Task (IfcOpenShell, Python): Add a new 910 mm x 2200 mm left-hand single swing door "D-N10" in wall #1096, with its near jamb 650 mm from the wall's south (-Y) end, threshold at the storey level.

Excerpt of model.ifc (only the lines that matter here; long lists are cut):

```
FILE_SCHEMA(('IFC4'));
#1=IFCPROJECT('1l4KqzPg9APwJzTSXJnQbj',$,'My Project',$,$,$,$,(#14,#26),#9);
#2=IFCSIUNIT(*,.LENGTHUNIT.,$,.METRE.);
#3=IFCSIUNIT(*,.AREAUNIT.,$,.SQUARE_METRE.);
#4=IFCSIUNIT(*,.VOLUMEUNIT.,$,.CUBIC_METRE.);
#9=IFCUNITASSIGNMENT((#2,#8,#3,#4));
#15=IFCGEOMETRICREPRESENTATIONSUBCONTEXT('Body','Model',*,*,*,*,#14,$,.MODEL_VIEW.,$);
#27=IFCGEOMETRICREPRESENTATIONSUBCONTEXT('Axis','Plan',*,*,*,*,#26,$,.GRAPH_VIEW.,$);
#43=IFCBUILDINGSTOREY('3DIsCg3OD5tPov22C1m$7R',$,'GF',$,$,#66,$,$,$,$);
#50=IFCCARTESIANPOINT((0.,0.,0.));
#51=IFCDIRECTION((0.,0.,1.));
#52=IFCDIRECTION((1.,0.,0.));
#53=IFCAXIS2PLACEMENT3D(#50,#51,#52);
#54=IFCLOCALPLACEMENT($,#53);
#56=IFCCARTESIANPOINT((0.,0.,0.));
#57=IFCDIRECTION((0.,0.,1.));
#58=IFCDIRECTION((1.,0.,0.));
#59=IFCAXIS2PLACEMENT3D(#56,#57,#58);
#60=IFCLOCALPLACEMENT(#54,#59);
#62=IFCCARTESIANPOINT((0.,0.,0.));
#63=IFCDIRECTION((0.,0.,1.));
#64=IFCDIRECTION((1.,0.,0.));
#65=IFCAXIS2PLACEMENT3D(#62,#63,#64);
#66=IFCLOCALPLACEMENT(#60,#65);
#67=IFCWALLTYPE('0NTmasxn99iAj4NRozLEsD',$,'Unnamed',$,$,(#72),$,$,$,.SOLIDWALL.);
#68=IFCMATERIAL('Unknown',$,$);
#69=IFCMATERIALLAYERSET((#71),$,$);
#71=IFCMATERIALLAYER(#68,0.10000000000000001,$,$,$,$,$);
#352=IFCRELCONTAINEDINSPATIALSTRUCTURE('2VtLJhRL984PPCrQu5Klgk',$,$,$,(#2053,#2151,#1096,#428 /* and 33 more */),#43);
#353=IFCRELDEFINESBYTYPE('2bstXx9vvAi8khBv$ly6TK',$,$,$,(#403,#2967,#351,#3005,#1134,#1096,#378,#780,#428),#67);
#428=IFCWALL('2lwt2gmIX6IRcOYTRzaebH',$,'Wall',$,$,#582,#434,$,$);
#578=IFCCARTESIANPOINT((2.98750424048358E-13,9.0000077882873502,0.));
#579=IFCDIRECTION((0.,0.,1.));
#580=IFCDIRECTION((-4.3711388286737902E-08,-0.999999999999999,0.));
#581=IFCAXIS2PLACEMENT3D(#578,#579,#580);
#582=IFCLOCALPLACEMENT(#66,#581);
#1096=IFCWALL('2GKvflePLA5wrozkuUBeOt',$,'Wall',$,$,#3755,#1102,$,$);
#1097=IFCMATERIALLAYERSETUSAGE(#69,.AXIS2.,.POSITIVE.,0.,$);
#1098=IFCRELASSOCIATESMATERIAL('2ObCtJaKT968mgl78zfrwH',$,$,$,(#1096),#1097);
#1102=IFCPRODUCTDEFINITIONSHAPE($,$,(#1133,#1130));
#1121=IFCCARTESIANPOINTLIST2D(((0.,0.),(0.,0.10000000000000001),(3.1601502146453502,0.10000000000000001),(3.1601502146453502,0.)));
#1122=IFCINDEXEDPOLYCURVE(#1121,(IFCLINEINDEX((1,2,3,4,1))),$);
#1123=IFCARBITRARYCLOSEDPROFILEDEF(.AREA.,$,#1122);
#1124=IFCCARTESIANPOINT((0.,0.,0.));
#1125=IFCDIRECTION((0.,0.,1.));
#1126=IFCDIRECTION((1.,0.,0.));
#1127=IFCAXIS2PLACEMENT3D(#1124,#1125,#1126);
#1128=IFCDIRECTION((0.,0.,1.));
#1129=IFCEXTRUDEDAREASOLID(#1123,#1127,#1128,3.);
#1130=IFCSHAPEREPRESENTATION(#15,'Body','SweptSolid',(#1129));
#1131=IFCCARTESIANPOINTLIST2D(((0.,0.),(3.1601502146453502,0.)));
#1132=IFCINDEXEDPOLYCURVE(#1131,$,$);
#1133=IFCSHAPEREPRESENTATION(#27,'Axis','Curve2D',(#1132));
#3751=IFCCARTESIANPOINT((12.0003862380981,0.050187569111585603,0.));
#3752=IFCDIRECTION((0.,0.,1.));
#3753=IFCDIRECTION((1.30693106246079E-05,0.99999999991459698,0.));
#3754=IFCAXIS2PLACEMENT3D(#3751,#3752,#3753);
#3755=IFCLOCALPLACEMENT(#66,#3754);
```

```python
import numpy as np
import ifcopenshell
import ifcopenshell.api.feature
import ifcopenshell.api.geometry
import ifcopenshell.api.root
import ifcopenshell.api.spatial
import ifcopenshell.geom
import ifcopenshell.util.element
import ifcopenshell.util.placement
import ifcopenshell.util.representation
import ifcopenshell.util.shape
import ifcopenshell.util.unit

model = ifcopenshell.open("model.ifc")
unit_scale = ifcopenshell.util.unit.calculate_unit_scale(model)
settings = ifcopenshell.geom.settings()


def volume(element):
    """Net volume in cubic metres, openings subtracted."""
    shape = ifcopenshell.geom.create_shape(settings, element)
    return ifcopenshell.util.shape.get_volume(shape.geometry)


wall = model.by_guid("2GKvflePLA5wrozkuUBeOt")
storey = ifcopenshell.util.element.get_container(wall, ifc_class="IfcBuildingStorey")
context = ifcopenshell.util.representation.get_context(model, "Model", "Body", "MODEL_VIEW")
before = volume(wall)

width, height, from_end, sill = 0.91, 2.2, 0.65, 0.0  # metres

# The wall runs along its own X axis, and the end named is its -X end.
wall_shape = ifcopenshell.geom.create_shape(settings, wall)
x, y, z = ifcopenshell.util.shape.get_vertices(wall_shape.geometry).T
start = x.min() + from_end
face, thickness = float(y.min()), float(y.max() - y.min())
wall_matrix = ifcopenshell.util.placement.get_local_placement(wall.ObjectPlacement)
level = ifcopenshell.util.placement.get_local_placement(storey.ObjectPlacement)[2, 3]


def in_wall(x, y):
    """Placement at x, y metres in the wall's axes, at sill height."""
    matrix = wall_matrix.copy()
    matrix[:, 3] = wall_matrix @ np.array([x / unit_scale, y / unit_scale, 0.0, 1.0])
    matrix[2, 3] = level + sill / unit_scale
    return matrix


# Opening: a box that overshoots both wall faces by 50 mm.
opening = ifcopenshell.api.root.create_entity(model, ifc_class="IfcOpeningElement", predefined_type="OPENING")
box = ifcopenshell.api.geometry.add_wall_representation(
    model, context=context, length=width, height=height, thickness=thickness + 0.1
)
ifcopenshell.api.geometry.assign_representation(model, product=opening, representation=box)
ifcopenshell.api.geometry.edit_object_placement(model, product=opening, matrix=in_wall(start, face - 0.05), is_si=False)
ifcopenshell.api.feature.add_feature(model, feature=opening, element=wall)

door = ifcopenshell.api.root.create_entity(model, ifc_class="IfcDoor", name="D-N10", predefined_type="DOOR")
door.OverallWidth, door.OverallHeight = width / unit_scale, height / unit_scale
door.OperationType = "SINGLE_SWING_LEFT"
body = ifcopenshell.api.geometry.add_door_representation(
    model,
    context=context,
    overall_width=door.OverallWidth,
    overall_height=door.OverallHeight,
    operation_type="SINGLE_SWING_LEFT",
    lining_properties={"LiningDepth": thickness / unit_scale, "ThresholdDepth": thickness / unit_scale},
)
ifcopenshell.api.geometry.assign_representation(model, product=door, representation=body)
ifcopenshell.api.spatial.assign_container(model, products=[door], relating_structure=storey)
ifcopenshell.api.feature.add_filling(model, opening=opening, element=door)

# The lining spans the wall, so the door starts at the wall face.
ifcopenshell.api.geometry.edit_object_placement(model, product=door, matrix=in_wall(start, face), is_si=False)

after = volume(wall)

print(f"wall volume {before:.3f} -> {after:.3f} m3")

model.write("model-out.ifc")
```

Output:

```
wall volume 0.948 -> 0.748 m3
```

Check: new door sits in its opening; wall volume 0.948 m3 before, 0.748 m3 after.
